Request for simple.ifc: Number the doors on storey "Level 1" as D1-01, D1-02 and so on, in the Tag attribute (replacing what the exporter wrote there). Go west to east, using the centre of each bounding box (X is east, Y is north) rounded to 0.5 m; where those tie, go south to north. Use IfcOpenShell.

First a look at what the model holds.

```python
import ifcopenshell
import ifcopenshell.util.element
import ifcopenshell.util.placement

model = ifcopenshell.open("simple.ifc")
print(model.schema)
storey = next(s for s in model.by_type("IfcBuildingStorey") if s.Name == "Level 1")
doors = [e for e in ifcopenshell.util.element.get_decomposition(storey) if e.is_a("IfcDoor")]
for e in sorted(doors, key=lambda e: e.id()):
    origin = ifcopenshell.util.placement.get_local_placement(e.ObjectPlacement)[:3, 3]
    print(e.id(), e.Tag, e.Name, origin.round(2) + 0.0, sep=" | ")
```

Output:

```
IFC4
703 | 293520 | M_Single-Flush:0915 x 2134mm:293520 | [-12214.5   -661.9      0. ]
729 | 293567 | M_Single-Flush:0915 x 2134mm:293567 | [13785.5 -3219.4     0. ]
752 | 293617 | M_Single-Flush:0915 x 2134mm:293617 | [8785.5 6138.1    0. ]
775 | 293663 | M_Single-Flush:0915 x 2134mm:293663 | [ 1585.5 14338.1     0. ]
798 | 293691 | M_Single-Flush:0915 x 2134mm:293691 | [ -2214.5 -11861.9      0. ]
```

```python
import ifcopenshell
import ifcopenshell.geom
import ifcopenshell.util.element
import ifcopenshell.util.shape

model = ifcopenshell.open("simple.ifc")
settings = ifcopenshell.geom.settings()
settings.set("use-world-coords", True)


def centre(element):
    shape = ifcopenshell.geom.create_shape(settings, element)
    return ifcopenshell.util.shape.get_bbox_centroid(shape.geometry)


storey = next(s for s in model.by_type("IfcBuildingStorey") if s.Name == "Level 1")
doors = [e for e in ifcopenshell.util.element.get_decomposition(storey) if e.is_a("IfcDoor")]

# Insertion points can sit at a corner or the storey origin, so sort by the geometry (in metres).
centres = {e: centre(e) for e in doors}
doors.sort(key=lambda e: (round(centres[e][0] / 0.5), centres[e][1]))

for i, e in enumerate(doors, start=1):
    number = f"D1-{i:02d}"
    e.Tag = number
    print(e.id(), number)

model.write("simple_updated.ifc")
```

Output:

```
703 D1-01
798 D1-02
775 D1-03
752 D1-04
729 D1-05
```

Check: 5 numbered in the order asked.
